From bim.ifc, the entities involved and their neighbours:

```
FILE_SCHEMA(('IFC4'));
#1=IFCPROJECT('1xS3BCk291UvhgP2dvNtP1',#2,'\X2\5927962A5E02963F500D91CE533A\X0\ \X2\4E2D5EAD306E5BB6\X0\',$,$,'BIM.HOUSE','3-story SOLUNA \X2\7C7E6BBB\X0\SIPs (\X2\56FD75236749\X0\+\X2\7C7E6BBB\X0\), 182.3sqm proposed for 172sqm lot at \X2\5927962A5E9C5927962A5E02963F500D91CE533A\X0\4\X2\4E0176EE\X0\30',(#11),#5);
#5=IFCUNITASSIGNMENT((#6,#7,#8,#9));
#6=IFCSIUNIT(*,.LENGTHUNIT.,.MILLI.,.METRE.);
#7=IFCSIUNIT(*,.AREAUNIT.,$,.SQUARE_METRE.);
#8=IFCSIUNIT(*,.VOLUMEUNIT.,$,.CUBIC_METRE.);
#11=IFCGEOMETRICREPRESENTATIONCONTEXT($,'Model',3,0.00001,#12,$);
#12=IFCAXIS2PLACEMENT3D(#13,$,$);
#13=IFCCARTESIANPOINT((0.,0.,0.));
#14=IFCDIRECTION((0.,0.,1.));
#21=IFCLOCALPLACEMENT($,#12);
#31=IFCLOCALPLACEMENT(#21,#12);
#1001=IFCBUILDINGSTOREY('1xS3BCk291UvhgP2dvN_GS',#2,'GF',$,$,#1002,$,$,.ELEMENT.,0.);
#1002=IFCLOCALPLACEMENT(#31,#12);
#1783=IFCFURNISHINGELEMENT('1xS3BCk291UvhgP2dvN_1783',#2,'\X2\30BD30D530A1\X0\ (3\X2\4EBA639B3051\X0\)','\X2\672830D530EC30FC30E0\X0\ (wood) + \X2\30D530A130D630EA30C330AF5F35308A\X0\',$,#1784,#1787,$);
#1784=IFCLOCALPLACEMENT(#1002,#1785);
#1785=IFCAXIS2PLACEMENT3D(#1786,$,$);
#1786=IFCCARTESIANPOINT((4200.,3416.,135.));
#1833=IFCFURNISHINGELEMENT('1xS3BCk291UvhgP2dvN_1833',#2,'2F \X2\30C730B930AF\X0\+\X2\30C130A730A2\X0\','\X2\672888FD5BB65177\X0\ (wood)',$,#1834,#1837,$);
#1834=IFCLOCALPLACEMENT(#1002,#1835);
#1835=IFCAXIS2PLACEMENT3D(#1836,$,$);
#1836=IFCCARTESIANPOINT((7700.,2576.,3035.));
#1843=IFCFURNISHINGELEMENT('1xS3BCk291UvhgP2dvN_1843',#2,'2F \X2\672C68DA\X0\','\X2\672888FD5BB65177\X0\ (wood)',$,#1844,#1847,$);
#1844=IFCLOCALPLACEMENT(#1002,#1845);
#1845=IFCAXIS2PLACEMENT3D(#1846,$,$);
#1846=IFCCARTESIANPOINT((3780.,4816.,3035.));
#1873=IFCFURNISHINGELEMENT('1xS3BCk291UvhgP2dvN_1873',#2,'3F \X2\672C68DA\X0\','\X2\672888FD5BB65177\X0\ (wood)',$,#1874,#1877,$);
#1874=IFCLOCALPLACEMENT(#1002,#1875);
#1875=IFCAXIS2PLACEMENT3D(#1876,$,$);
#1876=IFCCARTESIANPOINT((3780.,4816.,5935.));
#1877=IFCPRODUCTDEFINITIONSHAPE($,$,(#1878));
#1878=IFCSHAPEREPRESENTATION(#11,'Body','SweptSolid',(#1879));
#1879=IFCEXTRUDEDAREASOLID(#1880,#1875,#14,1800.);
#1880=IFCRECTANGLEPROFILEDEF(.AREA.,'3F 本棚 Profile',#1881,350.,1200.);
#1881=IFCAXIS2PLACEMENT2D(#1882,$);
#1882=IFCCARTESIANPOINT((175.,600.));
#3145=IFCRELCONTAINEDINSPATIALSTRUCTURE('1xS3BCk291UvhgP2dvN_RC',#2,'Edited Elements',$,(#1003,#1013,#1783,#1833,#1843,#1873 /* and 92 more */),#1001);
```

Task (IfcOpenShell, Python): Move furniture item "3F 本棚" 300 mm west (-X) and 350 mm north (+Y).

```python
import ifcopenshell
import ifcopenshell.api.geometry
import ifcopenshell.util.placement
import ifcopenshell.util.unit

model = ifcopenshell.open("bim.ifc")
unit_scale = ifcopenshell.util.unit.calculate_unit_scale(model)

item = model.by_guid("1xS3BCk291UvhgP2dvN_1873")
matrix = ifcopenshell.util.placement.get_local_placement(item.ObjectPlacement)
matrix[0, 3] -= 0.3 / unit_scale
matrix[1, 3] += 0.35 / unit_scale
ifcopenshell.api.geometry.edit_object_placement(model, product=item, matrix=matrix, is_si=False)

print(ifcopenshell.util.placement.get_local_placement(item.ObjectPlacement).round(3) + 0.0)

model.write("bim-out.ifc")
```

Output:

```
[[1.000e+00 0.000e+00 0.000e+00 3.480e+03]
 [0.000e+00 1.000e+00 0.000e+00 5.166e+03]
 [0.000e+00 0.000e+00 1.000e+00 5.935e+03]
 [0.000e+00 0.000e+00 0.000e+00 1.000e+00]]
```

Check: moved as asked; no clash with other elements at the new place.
